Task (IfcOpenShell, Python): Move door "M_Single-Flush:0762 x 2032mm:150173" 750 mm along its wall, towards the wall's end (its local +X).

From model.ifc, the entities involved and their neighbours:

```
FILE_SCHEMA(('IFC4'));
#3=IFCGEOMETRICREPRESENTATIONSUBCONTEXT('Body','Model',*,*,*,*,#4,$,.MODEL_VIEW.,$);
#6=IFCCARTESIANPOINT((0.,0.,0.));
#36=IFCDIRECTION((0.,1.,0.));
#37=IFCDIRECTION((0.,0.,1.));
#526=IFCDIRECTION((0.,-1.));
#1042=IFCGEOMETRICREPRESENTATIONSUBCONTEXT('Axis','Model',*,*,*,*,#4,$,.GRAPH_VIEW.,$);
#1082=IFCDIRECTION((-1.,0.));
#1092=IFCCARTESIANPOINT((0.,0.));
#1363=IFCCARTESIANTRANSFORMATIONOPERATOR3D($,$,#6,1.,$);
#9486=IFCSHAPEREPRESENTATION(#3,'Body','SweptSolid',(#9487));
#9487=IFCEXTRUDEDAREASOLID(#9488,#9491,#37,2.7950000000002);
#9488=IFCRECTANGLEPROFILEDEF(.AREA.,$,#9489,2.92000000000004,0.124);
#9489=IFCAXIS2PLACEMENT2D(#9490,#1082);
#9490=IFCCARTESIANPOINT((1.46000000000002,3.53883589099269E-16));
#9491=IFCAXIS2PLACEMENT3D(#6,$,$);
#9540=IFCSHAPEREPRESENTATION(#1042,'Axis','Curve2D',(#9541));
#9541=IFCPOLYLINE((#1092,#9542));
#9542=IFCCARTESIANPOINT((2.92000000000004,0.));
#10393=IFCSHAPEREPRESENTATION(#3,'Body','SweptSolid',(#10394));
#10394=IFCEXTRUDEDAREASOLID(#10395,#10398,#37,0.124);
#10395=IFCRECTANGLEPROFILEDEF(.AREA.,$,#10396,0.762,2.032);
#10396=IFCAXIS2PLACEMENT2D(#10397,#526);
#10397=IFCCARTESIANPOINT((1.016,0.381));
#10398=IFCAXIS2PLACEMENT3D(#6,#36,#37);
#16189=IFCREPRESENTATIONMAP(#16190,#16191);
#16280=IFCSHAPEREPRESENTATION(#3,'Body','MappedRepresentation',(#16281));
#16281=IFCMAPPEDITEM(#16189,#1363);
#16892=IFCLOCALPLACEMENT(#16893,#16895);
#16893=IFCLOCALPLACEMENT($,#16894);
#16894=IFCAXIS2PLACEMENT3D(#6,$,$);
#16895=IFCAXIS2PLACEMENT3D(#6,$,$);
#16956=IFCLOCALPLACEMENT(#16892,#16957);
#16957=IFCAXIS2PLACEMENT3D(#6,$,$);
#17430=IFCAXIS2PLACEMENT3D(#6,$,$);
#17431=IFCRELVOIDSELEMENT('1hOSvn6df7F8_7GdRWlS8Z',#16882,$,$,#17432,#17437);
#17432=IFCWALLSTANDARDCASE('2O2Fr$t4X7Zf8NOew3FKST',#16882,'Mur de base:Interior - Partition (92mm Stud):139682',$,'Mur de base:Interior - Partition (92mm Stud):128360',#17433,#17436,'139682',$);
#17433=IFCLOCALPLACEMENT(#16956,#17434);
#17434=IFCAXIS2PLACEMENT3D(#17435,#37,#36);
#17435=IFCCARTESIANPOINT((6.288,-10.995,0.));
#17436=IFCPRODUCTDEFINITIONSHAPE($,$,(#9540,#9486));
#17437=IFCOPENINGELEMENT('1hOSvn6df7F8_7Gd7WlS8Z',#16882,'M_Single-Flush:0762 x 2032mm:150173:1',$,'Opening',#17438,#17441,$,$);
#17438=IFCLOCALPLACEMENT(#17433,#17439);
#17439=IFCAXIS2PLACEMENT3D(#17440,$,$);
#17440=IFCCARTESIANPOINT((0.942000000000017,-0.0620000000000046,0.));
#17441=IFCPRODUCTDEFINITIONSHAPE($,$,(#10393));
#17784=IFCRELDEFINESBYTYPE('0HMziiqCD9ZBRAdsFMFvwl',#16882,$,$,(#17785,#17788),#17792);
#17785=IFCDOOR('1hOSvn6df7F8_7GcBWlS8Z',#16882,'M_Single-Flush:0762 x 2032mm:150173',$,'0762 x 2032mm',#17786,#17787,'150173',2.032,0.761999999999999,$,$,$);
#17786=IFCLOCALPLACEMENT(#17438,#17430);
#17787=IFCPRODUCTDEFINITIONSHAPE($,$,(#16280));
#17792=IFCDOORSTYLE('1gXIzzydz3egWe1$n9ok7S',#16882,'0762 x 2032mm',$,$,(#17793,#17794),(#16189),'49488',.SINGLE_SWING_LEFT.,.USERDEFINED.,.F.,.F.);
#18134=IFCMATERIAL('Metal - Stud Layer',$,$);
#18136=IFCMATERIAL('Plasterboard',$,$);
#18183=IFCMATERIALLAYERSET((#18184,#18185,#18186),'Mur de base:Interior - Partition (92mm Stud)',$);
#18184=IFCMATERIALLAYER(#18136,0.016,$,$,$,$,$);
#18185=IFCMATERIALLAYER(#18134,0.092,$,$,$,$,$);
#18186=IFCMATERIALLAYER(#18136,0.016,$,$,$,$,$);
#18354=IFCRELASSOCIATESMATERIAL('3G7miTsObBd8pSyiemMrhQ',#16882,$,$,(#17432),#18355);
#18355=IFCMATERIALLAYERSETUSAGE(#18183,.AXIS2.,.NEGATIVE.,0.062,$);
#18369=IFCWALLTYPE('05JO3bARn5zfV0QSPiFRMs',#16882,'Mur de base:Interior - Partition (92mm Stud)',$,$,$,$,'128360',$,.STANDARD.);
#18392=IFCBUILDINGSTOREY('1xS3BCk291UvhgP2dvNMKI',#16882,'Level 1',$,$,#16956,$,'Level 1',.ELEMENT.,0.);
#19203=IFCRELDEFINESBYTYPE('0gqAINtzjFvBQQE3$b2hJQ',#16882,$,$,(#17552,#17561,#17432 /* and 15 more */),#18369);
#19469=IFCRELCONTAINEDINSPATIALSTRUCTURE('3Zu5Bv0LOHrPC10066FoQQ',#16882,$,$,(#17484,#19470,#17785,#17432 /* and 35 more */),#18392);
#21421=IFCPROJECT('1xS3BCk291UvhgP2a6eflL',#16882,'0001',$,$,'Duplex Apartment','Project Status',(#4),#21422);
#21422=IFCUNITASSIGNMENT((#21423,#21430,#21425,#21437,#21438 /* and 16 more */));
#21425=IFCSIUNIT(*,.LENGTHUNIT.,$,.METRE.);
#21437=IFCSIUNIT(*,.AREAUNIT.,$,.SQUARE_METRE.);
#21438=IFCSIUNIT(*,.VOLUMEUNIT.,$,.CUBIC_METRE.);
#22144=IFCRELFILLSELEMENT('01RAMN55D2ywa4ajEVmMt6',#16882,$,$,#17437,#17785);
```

```python
import ifcopenshell
import ifcopenshell.api.geometry
import ifcopenshell.util.placement
import ifcopenshell.util.unit

model = ifcopenshell.open("model.ifc")
unit_scale = ifcopenshell.util.unit.calculate_unit_scale(model)

door = model.by_guid("1hOSvn6df7F8_7GcBWlS8Z")
opening = door.FillsVoids[0].RelatingOpeningElement
wall = opening.VoidsElements[0].RelatingBuildingElement

wall_matrix = ifcopenshell.util.placement.get_local_placement(wall.ObjectPlacement)
shift = wall_matrix[:3, 0] * 0.75 / unit_scale
before = ifcopenshell.util.placement.get_local_placement(door.ObjectPlacement)[:3, 3].copy()

# The door is placed relative to its opening, so it follows when the opening moves.
matrix = ifcopenshell.util.placement.get_local_placement(opening.ObjectPlacement)
matrix[:3, 3] += shift
ifcopenshell.api.geometry.edit_object_placement(
    model, product=opening, matrix=matrix, is_si=False, should_transform_children=True
)

after = ifcopenshell.util.placement.get_local_placement(door.ObjectPlacement)[:3, 3]
print("door moved by", (after - before).round(3) + 0.0)

model.write("model-out.ifc")
```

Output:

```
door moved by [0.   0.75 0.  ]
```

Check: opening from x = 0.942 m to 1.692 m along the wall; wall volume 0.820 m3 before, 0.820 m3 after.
